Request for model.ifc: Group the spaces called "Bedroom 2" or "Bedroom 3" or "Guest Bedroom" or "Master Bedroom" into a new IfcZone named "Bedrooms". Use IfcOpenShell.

First a look at what the model holds.

```python
import ifcopenshell

model = ifcopenshell.open("model.ifc")
print(model.schema)
seen = {}
for space in model.by_type("IfcSpace"):
    seen[space.LongName] = seen.get(space.LongName, 0) + 1
for name, count in sorted(seen.items(), key=str):
    print(count, "x", name)
print("zones:", [z.Name for z in model.by_type("IfcZone")][:20])
```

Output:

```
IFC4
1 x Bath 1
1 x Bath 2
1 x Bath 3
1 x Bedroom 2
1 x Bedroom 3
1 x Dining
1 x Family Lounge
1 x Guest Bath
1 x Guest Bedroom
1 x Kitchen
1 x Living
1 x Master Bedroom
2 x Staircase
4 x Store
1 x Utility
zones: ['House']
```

```python
import ifcopenshell
import ifcopenshell.api.group
import ifcopenshell.api.root

model = ifcopenshell.open("model.ifc")

names = {"Bedroom 2", "Bedroom 3", "Guest Bedroom", "Master Bedroom"}
spaces = [s for s in model.by_type("IfcSpace") if s.LongName in names]

zone = ifcopenshell.api.root.create_entity(model, ifc_class="IfcZone", name="Bedrooms")
ifcopenshell.api.group.assign_group(model, products=spaces, group=zone)
print(len(spaces), "spaces in", zone.Name)

model.write("model_edited.ifc")
```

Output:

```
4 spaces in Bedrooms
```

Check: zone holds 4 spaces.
